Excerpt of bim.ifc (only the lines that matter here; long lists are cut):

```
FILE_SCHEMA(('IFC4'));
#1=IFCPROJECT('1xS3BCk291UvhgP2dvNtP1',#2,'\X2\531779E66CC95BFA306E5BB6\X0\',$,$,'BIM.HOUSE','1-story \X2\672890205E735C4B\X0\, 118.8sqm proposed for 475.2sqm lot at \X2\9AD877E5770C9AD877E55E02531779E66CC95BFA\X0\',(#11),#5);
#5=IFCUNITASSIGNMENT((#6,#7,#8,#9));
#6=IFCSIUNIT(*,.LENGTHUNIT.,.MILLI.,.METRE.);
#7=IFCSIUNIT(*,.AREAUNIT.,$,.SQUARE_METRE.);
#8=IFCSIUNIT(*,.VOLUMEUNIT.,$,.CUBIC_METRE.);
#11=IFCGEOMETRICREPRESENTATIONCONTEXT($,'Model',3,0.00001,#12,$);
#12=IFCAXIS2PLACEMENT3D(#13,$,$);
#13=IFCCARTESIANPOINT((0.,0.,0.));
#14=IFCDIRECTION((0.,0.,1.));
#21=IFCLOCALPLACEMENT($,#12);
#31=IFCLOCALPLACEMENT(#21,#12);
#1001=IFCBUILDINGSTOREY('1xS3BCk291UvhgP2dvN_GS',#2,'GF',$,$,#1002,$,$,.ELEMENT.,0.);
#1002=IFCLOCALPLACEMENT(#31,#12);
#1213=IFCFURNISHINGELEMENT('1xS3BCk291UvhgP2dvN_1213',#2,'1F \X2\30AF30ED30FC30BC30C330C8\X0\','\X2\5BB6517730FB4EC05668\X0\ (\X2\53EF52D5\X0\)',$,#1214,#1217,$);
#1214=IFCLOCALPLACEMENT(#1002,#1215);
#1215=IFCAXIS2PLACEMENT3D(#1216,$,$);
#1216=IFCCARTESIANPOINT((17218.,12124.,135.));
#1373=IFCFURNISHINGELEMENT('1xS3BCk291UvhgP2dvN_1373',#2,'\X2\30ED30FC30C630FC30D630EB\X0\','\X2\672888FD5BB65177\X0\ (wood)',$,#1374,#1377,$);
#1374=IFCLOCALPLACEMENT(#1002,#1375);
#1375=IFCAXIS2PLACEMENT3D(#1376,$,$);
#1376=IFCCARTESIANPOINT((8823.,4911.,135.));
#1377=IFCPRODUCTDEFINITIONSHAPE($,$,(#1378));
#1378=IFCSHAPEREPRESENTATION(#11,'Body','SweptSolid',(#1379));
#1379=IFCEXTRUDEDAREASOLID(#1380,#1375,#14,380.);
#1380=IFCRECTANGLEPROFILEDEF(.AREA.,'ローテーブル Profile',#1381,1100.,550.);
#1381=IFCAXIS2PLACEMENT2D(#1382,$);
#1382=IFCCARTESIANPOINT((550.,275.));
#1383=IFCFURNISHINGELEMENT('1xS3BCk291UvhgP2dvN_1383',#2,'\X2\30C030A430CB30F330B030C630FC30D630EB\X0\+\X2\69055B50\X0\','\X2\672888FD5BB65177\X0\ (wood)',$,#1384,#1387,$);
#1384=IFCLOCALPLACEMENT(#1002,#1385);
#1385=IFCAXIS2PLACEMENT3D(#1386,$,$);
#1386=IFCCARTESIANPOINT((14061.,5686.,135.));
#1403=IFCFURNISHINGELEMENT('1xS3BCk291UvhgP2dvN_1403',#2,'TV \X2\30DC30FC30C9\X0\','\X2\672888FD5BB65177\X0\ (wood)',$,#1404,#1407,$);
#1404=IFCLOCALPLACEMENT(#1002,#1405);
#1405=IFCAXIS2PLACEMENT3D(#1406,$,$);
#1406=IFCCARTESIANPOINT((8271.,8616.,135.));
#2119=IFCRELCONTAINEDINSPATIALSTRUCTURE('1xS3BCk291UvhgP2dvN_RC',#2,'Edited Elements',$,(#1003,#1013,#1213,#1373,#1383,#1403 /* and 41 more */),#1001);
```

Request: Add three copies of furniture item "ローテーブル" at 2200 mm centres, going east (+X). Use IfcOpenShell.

```python
import numpy as np
import ifcopenshell
import ifcopenshell.api.geometry
import ifcopenshell.api.root
import ifcopenshell.util.element
import ifcopenshell.util.placement
import ifcopenshell.util.unit

model = ifcopenshell.open("bim.ifc")
unit_scale = ifcopenshell.util.unit.calculate_unit_scale(model)


def reuse_history(source, copy):
    """copy_class also copies each property set's owner history, people and application; keep the originals."""
    for rel in copy.IsDefinedBy:
        if rel.is_a("IfcRelDefinesByProperties") and (history := rel.RelatingPropertyDefinition.OwnerHistory):
            rel.RelatingPropertyDefinition.OwnerHistory = source.OwnerHistory
            ifcopenshell.util.element.remove_deep2(model, history)


source = model.by_id(1373)
base = ifcopenshell.util.placement.get_local_placement(source.ObjectPlacement)
step = np.array([1.0, 0.0, 0.0]) * 2.2 / unit_scale

for i in range(1, 4):
    copy = ifcopenshell.api.root.copy_class(model, product=source)
    copy.Representation = ifcopenshell.util.element.copy_deep(
        model, source.Representation, exclude=["IfcGeometricRepresentationContext", "IfcRepresentationMap"]
    )
    reuse_history(source, copy)
    matrix = base.copy()
    matrix[:3, 3] += i * step
    print("added at", matrix[:3, 3].round(3) + 0.0)
    ifcopenshell.api.geometry.edit_object_placement(model, product=copy, matrix=matrix, is_si=False)

model.write("bim_updated.ifc")
```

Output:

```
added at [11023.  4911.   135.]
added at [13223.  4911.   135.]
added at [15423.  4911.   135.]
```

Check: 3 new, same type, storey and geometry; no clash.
